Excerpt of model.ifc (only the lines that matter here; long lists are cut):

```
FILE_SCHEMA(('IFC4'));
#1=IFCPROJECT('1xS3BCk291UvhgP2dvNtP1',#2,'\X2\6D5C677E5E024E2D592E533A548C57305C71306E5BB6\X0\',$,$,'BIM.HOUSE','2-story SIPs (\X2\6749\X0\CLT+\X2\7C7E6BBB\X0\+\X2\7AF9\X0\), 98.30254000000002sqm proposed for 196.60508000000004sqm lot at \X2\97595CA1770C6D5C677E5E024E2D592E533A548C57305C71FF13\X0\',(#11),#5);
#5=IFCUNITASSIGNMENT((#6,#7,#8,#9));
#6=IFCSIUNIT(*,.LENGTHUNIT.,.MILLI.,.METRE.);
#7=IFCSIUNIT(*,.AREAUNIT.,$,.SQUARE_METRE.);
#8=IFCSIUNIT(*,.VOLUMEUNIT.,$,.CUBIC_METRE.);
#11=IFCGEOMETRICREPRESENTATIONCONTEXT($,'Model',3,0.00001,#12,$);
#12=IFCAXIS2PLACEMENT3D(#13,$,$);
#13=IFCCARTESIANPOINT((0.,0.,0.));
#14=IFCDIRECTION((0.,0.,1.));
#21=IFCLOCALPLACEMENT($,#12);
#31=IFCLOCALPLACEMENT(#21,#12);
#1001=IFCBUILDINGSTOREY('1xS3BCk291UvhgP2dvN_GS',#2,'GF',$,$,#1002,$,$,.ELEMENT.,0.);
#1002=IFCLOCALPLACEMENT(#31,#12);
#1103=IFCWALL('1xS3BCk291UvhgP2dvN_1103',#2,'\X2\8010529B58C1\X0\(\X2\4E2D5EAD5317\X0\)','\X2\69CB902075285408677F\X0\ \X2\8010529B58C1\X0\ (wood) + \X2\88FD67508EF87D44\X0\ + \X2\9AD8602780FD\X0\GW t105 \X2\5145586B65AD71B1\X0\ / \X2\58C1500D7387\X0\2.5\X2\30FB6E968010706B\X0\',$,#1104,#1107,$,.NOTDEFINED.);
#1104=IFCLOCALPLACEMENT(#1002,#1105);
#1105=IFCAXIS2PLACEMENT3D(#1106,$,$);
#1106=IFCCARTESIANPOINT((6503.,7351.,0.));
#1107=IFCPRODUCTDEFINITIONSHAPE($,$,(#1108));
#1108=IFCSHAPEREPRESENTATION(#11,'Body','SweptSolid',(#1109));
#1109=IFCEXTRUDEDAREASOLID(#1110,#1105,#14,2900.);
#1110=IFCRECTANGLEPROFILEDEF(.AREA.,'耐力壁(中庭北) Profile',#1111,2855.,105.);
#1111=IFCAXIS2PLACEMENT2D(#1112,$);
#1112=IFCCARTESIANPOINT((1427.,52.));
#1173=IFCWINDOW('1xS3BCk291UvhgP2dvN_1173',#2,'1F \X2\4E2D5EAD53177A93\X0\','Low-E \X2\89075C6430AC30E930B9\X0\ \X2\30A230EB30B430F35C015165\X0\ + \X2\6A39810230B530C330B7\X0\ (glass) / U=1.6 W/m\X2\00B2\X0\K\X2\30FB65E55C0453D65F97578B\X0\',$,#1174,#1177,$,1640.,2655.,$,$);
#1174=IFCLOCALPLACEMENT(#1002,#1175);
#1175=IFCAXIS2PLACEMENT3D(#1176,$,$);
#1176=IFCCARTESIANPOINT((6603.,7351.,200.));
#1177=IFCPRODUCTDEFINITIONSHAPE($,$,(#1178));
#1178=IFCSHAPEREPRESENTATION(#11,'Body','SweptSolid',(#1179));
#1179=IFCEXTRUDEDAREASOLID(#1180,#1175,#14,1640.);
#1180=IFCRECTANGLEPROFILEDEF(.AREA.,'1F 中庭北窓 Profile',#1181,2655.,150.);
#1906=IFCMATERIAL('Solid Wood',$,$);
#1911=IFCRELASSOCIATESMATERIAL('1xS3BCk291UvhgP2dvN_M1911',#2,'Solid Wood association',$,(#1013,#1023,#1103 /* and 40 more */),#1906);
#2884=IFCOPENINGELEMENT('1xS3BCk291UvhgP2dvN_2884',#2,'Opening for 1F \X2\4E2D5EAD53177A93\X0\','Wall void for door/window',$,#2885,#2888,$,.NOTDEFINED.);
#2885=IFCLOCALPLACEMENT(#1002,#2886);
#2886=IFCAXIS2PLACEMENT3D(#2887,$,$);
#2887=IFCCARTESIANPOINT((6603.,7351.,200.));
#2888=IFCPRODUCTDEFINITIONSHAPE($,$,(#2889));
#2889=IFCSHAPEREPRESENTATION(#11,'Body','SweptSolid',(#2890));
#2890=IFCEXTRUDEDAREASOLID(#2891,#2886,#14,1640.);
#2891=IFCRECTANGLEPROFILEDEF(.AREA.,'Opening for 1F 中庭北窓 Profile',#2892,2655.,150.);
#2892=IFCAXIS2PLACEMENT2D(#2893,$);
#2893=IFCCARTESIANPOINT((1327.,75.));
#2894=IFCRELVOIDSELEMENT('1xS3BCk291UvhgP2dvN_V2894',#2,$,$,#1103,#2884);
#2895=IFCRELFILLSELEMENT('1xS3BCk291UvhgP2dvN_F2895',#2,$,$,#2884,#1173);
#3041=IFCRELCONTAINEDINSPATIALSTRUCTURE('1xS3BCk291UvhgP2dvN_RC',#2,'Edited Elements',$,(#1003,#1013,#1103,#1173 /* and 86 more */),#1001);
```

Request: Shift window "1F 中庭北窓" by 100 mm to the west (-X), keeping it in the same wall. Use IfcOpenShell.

```python
import ifcopenshell
import ifcopenshell.api.geometry
import ifcopenshell.util.placement
import ifcopenshell.util.unit

model = ifcopenshell.open("model.ifc")
unit_scale = ifcopenshell.util.unit.calculate_unit_scale(model)

window = model.by_guid("1xS3BCk291UvhgP2dvN_1173")
opening = window.FillsVoids[0].RelatingOpeningElement
wall = opening.VoidsElements[0].RelatingBuildingElement

wall_matrix = ifcopenshell.util.placement.get_local_placement(wall.ObjectPlacement)
shift = wall_matrix[:3, 0] * -0.1 / unit_scale
before = ifcopenshell.util.placement.get_local_placement(window.ObjectPlacement)[:3, 3].copy()

# The window is not placed relative to its opening, so move both.
for product in (opening, window):
    matrix = ifcopenshell.util.placement.get_local_placement(product.ObjectPlacement)
    matrix[:3, 3] += shift
    ifcopenshell.api.geometry.edit_object_placement(model, product=product, matrix=matrix, is_si=False)

after = ifcopenshell.util.placement.get_local_placement(window.ObjectPlacement)[:3, 3]
print("window moved by", (after - before).round(3) + 0.0)

model.write("model_edited.ifc")
```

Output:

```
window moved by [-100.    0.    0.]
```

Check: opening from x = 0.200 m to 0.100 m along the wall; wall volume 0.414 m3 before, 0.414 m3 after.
